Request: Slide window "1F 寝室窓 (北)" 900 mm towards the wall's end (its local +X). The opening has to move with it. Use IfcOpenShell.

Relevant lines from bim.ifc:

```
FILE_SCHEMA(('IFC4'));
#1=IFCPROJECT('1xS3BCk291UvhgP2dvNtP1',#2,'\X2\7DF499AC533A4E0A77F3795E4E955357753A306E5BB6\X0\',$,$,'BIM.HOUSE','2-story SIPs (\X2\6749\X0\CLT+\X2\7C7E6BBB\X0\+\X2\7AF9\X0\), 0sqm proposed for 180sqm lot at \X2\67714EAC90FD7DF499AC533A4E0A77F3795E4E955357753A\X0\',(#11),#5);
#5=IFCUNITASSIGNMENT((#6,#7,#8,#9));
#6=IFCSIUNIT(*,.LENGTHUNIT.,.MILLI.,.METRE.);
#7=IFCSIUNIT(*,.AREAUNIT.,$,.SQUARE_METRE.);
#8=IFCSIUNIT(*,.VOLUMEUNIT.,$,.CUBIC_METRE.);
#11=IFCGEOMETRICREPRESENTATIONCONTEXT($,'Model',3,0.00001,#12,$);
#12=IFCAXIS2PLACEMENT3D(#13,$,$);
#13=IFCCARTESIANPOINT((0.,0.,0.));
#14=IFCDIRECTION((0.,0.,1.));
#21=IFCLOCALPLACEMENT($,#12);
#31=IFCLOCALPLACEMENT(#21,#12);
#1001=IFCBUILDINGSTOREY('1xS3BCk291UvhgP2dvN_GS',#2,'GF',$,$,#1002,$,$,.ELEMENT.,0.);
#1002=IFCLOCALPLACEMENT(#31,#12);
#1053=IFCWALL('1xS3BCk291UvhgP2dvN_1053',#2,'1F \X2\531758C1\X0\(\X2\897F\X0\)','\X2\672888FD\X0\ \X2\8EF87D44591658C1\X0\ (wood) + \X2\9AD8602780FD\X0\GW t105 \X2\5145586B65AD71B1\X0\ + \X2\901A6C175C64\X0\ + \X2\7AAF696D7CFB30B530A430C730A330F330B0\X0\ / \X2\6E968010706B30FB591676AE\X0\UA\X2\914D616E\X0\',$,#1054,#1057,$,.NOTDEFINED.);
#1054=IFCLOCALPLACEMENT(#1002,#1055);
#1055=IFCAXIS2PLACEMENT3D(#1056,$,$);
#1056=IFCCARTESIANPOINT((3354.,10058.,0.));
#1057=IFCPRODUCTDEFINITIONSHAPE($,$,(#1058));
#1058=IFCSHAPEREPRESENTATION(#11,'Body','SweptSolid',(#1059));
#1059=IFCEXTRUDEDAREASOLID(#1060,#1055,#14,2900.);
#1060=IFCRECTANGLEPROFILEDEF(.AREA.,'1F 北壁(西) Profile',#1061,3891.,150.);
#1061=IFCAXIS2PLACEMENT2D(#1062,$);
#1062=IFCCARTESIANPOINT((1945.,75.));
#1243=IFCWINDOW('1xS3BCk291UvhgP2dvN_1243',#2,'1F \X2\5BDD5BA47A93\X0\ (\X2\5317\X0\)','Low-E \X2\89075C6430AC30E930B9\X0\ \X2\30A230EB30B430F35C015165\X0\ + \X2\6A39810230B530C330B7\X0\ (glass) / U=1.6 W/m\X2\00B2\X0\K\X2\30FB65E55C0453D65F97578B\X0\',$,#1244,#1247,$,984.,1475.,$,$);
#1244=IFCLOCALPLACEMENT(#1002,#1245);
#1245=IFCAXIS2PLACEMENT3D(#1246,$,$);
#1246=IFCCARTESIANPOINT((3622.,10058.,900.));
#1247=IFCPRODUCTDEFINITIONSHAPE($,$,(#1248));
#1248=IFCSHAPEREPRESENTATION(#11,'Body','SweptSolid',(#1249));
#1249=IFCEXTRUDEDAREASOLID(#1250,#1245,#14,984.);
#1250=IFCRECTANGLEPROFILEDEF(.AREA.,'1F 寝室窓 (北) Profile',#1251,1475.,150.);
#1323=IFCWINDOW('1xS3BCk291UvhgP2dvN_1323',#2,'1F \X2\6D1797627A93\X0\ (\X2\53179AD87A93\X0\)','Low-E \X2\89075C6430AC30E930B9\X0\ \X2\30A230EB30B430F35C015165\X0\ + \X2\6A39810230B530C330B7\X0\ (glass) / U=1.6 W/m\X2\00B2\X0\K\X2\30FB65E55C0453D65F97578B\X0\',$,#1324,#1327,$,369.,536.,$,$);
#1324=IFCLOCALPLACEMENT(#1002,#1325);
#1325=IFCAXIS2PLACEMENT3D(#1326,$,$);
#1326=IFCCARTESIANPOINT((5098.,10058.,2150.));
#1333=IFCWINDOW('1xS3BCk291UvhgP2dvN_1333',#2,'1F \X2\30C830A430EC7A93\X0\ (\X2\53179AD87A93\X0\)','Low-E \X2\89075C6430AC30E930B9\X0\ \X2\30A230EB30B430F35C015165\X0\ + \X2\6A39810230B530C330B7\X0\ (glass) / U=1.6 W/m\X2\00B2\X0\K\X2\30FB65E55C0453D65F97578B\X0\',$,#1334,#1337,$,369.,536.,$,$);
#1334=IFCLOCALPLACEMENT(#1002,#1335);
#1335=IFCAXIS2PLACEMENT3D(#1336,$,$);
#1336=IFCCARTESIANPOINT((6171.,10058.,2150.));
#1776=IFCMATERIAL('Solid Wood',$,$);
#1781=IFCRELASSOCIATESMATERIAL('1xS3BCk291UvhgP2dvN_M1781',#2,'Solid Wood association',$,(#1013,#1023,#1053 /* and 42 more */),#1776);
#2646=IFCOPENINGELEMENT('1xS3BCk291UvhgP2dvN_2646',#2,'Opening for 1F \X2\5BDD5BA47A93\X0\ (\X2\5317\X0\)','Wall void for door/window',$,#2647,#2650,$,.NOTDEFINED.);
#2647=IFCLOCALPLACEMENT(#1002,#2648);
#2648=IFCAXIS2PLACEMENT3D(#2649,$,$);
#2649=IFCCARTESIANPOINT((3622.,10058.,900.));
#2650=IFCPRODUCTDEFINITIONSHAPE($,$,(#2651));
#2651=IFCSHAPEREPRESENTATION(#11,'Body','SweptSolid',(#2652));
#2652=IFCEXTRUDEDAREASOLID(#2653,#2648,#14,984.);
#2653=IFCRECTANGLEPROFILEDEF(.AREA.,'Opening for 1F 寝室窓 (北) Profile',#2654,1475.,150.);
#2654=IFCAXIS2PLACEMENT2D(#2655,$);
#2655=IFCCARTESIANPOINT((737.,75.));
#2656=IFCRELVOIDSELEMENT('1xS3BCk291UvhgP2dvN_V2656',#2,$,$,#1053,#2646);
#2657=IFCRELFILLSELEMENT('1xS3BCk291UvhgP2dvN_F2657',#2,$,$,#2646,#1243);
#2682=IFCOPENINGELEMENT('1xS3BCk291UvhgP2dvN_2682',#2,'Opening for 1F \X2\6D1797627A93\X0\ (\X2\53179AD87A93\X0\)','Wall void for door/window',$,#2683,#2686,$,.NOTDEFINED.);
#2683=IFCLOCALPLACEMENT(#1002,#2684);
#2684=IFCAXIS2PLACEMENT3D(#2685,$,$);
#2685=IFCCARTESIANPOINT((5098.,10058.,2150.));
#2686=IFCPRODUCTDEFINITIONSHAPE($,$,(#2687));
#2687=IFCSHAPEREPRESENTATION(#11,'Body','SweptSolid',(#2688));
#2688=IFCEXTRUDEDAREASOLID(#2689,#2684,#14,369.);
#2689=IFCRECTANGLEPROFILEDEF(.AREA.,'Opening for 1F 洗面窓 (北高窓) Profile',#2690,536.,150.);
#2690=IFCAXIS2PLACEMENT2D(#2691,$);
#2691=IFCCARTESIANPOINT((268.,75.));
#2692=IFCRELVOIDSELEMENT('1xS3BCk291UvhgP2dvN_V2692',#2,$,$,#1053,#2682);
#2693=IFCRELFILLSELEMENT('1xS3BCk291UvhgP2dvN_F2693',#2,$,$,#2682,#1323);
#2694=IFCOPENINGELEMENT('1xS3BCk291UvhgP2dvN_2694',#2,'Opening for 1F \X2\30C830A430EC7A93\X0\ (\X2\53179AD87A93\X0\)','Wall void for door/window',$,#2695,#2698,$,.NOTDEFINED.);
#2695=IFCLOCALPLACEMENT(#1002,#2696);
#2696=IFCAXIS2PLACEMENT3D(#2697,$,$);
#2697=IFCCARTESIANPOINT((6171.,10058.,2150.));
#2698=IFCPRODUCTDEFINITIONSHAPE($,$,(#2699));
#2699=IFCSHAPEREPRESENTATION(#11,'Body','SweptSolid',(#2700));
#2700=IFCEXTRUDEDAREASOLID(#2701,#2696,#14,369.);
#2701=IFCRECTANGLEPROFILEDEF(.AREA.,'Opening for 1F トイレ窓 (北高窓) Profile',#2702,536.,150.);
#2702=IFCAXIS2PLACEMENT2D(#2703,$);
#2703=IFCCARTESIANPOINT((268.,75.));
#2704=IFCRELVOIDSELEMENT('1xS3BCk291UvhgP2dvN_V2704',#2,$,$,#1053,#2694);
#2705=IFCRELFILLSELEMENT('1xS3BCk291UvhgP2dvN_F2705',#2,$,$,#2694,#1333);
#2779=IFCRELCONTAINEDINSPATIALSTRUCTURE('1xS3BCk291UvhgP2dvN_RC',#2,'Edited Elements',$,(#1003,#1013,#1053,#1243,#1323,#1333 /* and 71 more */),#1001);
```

```python
import ifcopenshell
import ifcopenshell.api.geometry
import ifcopenshell.util.placement

model = ifcopenshell.open("bim.ifc")

window = model.by_guid("1xS3BCk291UvhgP2dvN_1243")
opening = window.FillsVoids[0].RelatingOpeningElement
wall = opening.VoidsElements[0].RelatingBuildingElement

wall_matrix = ifcopenshell.util.placement.get_local_placement(wall.ObjectPlacement)
shift = wall_matrix[:3, 0] * 900.0
before = ifcopenshell.util.placement.get_local_placement(window.ObjectPlacement)[:3, 3].copy()

# The window is not placed relative to its opening, so move both.
for product in (opening, window):
    matrix = ifcopenshell.util.placement.get_local_placement(product.ObjectPlacement)
    matrix[:3, 3] += shift
    ifcopenshell.api.geometry.edit_object_placement(model, product=product, matrix=matrix, is_si=False)

after = ifcopenshell.util.placement.get_local_placement(window.ObjectPlacement)[:3, 3]
print("window moved by", (after - before).round(3) + 0.0)

model.write("bim-out.ifc")
```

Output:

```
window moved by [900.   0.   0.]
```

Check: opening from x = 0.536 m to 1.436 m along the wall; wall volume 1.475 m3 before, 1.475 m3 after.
